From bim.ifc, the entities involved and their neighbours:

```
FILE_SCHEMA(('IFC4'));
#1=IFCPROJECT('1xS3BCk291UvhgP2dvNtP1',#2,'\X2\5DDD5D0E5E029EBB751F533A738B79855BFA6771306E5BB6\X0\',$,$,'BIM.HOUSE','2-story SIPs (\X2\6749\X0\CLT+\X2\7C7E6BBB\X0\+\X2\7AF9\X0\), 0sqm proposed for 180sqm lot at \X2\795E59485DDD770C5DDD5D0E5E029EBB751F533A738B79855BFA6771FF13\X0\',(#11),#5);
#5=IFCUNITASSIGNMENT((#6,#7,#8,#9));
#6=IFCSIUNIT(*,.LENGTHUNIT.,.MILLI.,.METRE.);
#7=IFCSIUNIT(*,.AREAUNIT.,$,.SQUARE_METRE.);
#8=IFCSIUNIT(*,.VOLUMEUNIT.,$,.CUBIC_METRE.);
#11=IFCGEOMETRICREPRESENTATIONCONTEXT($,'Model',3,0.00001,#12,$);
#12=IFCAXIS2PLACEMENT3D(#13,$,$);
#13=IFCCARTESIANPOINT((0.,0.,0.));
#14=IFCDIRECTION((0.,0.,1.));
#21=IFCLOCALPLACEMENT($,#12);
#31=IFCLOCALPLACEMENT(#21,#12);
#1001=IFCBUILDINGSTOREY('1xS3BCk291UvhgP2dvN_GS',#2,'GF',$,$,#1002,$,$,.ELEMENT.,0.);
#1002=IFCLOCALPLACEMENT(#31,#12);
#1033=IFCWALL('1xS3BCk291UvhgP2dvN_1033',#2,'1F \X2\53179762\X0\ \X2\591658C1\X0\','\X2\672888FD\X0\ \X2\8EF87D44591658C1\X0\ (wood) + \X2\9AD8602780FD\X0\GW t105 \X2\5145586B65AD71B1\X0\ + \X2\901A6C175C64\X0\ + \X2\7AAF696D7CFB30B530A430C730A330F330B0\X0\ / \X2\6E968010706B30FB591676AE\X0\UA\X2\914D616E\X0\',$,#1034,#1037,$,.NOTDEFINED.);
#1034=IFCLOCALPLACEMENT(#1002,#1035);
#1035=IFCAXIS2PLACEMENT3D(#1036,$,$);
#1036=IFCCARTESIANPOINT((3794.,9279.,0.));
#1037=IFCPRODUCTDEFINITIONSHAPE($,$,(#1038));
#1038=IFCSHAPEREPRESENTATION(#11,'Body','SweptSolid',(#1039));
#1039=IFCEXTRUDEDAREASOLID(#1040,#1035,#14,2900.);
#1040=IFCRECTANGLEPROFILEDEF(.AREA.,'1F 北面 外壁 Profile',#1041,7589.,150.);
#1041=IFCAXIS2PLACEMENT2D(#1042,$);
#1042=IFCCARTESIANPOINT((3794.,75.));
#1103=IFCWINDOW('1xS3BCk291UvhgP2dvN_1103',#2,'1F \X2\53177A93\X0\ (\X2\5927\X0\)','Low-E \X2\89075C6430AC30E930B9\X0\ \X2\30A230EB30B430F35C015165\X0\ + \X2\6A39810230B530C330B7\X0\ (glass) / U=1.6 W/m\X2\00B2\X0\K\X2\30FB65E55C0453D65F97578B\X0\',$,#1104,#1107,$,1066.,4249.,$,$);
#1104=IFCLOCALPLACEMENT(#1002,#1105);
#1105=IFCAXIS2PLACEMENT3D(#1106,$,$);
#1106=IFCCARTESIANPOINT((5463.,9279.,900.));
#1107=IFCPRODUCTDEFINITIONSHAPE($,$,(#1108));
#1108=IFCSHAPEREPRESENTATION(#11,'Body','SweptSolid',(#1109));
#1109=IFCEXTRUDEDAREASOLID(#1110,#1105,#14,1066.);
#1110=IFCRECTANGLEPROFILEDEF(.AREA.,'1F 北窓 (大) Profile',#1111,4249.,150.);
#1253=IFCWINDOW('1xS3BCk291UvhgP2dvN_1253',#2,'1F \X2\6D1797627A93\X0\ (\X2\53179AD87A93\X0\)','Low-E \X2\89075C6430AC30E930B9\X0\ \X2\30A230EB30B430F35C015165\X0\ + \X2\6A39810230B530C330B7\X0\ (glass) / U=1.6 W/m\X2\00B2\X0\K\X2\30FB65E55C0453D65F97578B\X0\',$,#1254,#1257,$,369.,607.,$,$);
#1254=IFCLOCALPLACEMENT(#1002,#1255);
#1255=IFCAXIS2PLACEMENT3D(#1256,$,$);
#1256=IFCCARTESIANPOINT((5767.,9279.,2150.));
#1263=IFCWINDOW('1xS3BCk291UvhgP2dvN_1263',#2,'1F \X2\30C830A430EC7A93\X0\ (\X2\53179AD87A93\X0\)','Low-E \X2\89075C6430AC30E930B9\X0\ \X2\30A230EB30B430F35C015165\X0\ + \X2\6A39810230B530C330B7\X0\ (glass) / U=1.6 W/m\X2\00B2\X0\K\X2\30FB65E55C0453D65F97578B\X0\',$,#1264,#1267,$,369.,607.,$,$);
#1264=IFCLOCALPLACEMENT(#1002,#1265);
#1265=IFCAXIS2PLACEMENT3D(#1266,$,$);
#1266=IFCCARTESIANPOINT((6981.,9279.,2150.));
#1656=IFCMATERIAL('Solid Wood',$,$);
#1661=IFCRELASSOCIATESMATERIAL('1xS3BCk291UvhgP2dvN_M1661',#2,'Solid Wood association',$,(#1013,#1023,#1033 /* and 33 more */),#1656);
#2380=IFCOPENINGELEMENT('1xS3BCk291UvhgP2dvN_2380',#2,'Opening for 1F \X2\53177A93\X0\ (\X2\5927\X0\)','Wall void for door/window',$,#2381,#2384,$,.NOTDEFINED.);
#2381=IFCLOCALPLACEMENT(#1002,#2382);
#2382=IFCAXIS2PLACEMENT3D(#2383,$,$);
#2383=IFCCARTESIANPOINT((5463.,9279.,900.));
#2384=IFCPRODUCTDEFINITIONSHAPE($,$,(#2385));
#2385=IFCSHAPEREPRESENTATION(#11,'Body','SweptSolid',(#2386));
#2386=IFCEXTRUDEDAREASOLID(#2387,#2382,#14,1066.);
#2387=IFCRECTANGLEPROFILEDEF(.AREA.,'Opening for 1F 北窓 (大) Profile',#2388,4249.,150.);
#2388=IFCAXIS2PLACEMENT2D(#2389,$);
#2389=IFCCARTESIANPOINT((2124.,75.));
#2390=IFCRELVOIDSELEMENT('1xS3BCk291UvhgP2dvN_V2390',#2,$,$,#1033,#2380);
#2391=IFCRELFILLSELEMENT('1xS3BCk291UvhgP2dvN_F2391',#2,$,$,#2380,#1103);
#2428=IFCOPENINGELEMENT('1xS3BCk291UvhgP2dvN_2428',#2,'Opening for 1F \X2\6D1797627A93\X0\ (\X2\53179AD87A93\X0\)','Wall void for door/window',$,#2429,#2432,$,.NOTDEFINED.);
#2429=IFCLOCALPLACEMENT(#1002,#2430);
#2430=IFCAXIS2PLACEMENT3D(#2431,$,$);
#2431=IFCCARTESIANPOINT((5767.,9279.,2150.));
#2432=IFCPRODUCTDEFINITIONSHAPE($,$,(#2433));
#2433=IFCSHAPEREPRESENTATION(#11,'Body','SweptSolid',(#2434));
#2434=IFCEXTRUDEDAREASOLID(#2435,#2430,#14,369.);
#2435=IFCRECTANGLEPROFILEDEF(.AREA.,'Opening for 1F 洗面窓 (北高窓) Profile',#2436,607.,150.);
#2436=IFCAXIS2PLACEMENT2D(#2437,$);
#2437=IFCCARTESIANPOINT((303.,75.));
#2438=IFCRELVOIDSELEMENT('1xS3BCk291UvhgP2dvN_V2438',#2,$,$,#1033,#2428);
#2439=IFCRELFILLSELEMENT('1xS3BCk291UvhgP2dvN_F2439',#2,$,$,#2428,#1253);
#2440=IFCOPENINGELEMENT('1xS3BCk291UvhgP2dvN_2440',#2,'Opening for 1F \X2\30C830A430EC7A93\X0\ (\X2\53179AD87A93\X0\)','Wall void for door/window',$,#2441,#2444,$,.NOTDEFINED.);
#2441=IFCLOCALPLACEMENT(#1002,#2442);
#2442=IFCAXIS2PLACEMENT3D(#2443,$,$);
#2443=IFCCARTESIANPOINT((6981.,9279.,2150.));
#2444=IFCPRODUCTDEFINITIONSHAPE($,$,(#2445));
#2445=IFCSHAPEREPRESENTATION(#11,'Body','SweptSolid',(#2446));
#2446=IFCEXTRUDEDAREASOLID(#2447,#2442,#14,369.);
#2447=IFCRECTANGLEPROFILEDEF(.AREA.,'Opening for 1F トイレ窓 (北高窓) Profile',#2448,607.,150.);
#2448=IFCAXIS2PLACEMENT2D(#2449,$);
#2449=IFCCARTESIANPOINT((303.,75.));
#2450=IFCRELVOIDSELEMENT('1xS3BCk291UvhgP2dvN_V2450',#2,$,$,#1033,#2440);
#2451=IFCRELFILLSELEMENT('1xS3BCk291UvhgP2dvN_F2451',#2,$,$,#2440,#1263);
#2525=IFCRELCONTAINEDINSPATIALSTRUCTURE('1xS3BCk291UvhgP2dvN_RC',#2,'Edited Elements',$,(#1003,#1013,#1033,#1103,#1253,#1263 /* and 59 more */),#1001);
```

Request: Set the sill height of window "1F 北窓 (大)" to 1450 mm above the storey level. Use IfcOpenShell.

```python
import numpy as np
import ifcopenshell
import ifcopenshell.api.geometry
import ifcopenshell.geom
import ifcopenshell.util.element
import ifcopenshell.util.placement
import ifcopenshell.util.shape
import ifcopenshell.util.unit

model = ifcopenshell.open("bim.ifc")
unit_scale = ifcopenshell.util.unit.calculate_unit_scale(model)

window = model.by_guid("1xS3BCk291UvhgP2dvN_1103")
opening = window.FillsVoids[0].RelatingOpeningElement
storey = ifcopenshell.util.element.get_container(window, ifc_class="IfcBuildingStorey")
level = ifcopenshell.util.placement.get_local_placement(storey.ObjectPlacement)[2, 3]

# The opening's origin need not be at the sill, so measure its lowest point.
shape = ifcopenshell.geom.create_shape(ifcopenshell.geom.settings(), opening)
bottom = ifcopenshell.util.shape.get_shape_bottom_elevation(shape, shape.geometry) / unit_scale
dz = level + 1450.0 - bottom

shift = np.array([0.0, 0.0, dz])
# The window is not placed relative to its opening, so move both.
for product in (opening, window):
    matrix = ifcopenshell.util.placement.get_local_placement(product.ObjectPlacement)
    matrix[:3, 3] += shift
    ifcopenshell.api.geometry.edit_object_placement(model, product=product, matrix=matrix, is_si=False)

print(f"moved by {dz * unit_scale:+.3f} m")

model.write("bim_rev.ifc")
```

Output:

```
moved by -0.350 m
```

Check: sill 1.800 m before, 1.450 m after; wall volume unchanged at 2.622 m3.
